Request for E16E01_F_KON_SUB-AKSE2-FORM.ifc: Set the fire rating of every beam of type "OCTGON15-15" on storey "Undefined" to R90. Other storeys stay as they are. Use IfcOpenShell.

First a look at what the model holds.

```python
import ifcopenshell
import ifcopenshell.util.element

model = ifcopenshell.open("E16E01_F_KON_SUB-AKSE2-FORM.ifc")
print(model.schema)
storey = next(s for s in model.by_type("IfcBuildingStorey") if s.Name == "Undefined")
beams = [e for e in ifcopenshell.util.element.get_decomposition(storey) if e.is_a("IfcBeam")]
seen = {}
for e in beams:
    element_type = ifcopenshell.util.element.get_type(e)
    key = (element_type.Name if element_type != e and element_type else None, ifcopenshell.util.element.get_pset(e, "Pset_BeamCommon", "FireRating"))
    seen[key] = seen.get(key, 0) + 1
for (name, value), count in sorted(seen.items(), key=str):
    print(count, "x", name, "|", value)
```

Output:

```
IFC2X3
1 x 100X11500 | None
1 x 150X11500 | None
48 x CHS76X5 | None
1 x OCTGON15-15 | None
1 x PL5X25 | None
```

```python
import ifcopenshell
import ifcopenshell.api.pset
import ifcopenshell.util.element

model = ifcopenshell.open("E16E01_F_KON_SUB-AKSE2-FORM.ifc")

storey = next(s for s in model.by_type("IfcBuildingStorey") if s.Name == "Undefined")
beams = [e for e in ifcopenshell.util.element.get_decomposition(storey) if e.is_a("IfcBeam")]

count = 0
for e in beams:
    element_type = ifcopenshell.util.element.get_type(e)
    if element_type in (None, e) or element_type.Name != "OCTGON15-15":
        continue
    # add_pset returns the element's existing set when there is one.
    pset = ifcopenshell.api.pset.add_pset(model, product=e, name="Pset_BeamCommon")
    ifcopenshell.api.pset.edit_pset(model, pset=pset, properties={"FireRating": "R90"})
    count += 1

print(count, "beams updated")

model.write("E16E01_F_KON_SUB-AKSE2-FORM_v2.ifc")
```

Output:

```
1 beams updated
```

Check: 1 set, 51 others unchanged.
